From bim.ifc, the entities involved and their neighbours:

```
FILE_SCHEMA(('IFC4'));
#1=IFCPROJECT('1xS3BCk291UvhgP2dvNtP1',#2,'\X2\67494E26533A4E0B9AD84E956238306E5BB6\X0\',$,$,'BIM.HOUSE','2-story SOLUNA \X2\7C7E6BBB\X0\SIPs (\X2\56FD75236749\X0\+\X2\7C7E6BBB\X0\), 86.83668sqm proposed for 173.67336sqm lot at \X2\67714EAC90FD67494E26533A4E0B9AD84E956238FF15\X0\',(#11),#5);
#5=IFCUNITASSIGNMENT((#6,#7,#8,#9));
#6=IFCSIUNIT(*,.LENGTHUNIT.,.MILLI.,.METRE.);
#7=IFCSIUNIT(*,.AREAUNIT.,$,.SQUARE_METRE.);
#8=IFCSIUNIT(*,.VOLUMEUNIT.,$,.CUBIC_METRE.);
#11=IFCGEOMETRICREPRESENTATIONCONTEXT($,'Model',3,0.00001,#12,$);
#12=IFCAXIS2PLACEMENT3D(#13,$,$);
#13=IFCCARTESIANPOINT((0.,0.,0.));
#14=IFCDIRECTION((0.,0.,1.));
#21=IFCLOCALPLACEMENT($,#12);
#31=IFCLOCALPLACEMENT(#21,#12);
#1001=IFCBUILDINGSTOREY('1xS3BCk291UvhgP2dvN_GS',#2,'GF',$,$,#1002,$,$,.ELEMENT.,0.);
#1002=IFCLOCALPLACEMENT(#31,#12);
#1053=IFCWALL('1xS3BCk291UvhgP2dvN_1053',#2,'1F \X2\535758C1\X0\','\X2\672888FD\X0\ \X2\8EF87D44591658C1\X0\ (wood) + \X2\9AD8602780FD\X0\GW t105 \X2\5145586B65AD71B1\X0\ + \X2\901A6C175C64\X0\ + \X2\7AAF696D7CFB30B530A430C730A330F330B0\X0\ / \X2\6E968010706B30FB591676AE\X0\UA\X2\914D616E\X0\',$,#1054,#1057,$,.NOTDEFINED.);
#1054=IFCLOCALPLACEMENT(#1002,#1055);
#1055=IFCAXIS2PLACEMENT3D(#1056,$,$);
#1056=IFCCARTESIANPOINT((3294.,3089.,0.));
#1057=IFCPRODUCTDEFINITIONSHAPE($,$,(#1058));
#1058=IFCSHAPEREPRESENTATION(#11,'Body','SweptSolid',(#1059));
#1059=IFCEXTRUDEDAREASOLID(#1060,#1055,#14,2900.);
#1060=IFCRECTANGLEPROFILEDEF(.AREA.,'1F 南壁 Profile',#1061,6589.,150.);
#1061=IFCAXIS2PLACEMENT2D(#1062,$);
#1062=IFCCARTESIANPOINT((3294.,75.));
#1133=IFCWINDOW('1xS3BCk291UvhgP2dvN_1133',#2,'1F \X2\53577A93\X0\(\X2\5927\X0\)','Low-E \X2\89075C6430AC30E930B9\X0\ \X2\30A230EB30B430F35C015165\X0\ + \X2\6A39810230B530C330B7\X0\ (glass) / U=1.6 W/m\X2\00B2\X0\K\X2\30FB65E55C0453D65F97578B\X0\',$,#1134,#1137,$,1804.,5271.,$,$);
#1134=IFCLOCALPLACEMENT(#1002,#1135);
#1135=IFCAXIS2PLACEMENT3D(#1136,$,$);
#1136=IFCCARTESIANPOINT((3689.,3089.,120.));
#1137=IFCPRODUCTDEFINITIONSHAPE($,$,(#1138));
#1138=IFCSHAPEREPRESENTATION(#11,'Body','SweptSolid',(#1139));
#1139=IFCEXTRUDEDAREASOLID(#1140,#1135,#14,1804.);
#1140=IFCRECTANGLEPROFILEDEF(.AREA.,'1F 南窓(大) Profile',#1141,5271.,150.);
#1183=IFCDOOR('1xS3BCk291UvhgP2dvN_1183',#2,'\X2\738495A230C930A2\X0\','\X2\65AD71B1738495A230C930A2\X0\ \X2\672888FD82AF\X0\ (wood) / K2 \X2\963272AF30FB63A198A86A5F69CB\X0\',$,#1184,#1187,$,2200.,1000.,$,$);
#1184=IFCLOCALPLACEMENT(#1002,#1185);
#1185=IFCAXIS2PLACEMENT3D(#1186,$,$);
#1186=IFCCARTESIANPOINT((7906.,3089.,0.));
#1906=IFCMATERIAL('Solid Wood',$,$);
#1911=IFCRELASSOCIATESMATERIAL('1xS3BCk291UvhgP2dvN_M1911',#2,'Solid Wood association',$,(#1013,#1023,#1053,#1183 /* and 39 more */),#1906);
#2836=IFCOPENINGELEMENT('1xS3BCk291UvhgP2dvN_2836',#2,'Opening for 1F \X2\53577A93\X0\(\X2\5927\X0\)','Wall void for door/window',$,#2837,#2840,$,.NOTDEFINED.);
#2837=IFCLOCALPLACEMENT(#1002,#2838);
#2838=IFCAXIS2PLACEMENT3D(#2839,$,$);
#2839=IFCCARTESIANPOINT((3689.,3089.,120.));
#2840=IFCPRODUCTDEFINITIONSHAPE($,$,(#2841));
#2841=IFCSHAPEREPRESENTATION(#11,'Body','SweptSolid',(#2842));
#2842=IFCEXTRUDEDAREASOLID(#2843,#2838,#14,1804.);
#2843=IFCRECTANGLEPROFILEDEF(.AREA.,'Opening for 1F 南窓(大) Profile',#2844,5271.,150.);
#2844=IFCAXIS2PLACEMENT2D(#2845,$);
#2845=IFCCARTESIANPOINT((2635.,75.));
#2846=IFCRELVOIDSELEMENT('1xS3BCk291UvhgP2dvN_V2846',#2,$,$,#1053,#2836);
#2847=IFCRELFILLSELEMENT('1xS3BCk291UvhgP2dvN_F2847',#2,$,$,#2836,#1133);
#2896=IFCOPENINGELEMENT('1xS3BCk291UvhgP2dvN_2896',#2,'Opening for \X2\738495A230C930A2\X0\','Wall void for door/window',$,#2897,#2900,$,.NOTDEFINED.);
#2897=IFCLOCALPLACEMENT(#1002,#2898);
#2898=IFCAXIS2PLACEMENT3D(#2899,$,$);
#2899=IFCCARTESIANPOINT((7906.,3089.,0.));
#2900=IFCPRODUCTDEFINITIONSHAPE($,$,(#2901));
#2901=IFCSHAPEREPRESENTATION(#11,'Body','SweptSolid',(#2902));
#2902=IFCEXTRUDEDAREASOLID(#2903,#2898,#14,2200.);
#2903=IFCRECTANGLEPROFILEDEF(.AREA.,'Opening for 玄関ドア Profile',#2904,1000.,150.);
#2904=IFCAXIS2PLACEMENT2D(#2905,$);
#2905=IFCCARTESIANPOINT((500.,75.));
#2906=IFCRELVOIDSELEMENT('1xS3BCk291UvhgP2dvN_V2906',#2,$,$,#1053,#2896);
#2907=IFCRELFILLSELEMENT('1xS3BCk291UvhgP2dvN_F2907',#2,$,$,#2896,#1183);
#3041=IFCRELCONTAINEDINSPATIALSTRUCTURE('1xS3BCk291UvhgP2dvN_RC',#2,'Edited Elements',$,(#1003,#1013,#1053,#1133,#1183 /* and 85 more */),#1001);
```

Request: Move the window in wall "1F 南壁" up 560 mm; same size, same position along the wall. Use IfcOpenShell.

```python
import numpy as np
import ifcopenshell
import ifcopenshell.api.geometry
import ifcopenshell.util.placement
import ifcopenshell.util.unit

model = ifcopenshell.open("bim.ifc")
unit_scale = ifcopenshell.util.unit.calculate_unit_scale(model)

window = model.by_guid("1xS3BCk291UvhgP2dvN_1133")
opening = window.FillsVoids[0].RelatingOpeningElement
dz = 0.56 / unit_scale

shift = np.array([0.0, 0.0, dz])
# The window is not placed relative to its opening, so move both.
for product in (opening, window):
    matrix = ifcopenshell.util.placement.get_local_placement(product.ObjectPlacement)
    matrix[:3, 3] += shift
    ifcopenshell.api.geometry.edit_object_placement(model, product=product, matrix=matrix, is_si=False)

print(f"moved by {dz * unit_scale:+.3f} m")

model.write("bim_rev.ifc")
```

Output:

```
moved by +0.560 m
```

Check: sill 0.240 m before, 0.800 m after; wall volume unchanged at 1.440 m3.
